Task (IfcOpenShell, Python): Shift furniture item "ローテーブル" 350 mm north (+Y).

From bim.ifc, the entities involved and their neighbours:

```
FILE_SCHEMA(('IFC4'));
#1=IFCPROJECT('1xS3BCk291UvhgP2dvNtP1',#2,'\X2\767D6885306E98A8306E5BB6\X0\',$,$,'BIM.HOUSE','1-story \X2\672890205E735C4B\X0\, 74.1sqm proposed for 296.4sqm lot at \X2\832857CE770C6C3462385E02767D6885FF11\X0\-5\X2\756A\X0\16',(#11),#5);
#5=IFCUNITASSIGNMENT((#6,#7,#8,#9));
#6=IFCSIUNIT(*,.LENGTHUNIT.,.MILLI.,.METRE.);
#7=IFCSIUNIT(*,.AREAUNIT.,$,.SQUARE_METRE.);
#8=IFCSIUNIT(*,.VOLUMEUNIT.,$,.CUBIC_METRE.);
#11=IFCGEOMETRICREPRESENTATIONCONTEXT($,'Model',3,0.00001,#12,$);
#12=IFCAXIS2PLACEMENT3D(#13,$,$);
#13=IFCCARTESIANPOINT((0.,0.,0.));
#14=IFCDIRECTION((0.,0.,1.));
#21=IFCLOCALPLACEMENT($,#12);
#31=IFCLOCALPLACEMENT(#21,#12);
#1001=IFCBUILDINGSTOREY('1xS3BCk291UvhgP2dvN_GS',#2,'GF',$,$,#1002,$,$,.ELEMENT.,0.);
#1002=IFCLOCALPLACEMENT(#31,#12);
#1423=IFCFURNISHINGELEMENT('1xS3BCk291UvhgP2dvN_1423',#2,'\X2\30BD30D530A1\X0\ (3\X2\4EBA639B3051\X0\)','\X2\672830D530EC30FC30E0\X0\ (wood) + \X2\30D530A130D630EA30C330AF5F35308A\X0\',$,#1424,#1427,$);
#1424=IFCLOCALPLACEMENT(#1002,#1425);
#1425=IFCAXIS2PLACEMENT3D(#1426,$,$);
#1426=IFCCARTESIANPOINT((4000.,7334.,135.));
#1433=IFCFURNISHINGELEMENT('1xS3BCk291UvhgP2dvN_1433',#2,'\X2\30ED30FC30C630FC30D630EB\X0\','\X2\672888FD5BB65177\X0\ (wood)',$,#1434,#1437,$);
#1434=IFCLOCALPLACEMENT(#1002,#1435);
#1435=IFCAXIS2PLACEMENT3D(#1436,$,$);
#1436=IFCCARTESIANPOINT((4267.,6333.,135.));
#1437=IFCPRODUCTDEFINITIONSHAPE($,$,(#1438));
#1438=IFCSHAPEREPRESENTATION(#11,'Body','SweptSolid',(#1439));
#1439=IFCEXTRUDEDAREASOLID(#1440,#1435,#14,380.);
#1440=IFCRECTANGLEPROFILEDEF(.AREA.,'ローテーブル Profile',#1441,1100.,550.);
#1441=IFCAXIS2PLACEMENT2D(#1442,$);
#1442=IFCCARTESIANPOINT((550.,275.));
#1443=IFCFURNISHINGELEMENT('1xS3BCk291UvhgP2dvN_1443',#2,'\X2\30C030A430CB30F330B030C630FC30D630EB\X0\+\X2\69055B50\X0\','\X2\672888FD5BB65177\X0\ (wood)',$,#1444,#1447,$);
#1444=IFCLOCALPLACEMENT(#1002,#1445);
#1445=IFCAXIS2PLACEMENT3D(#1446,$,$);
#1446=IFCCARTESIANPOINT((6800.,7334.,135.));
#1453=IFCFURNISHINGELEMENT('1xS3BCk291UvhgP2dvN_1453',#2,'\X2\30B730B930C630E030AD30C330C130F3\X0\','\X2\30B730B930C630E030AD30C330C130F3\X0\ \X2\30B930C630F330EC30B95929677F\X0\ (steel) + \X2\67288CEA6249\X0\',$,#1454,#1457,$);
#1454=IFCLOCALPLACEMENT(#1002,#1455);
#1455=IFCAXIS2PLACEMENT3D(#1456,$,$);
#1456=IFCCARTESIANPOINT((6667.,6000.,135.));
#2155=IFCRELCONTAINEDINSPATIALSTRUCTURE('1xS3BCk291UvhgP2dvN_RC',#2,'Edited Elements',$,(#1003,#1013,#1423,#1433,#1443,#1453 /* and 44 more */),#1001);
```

```python
import ifcopenshell
import ifcopenshell.api.geometry
import ifcopenshell.util.placement
import ifcopenshell.util.unit

model = ifcopenshell.open("bim.ifc")
unit_scale = ifcopenshell.util.unit.calculate_unit_scale(model)

item = model.by_guid("1xS3BCk291UvhgP2dvN_1433")
matrix = ifcopenshell.util.placement.get_local_placement(item.ObjectPlacement)
matrix[1, 3] += 0.35 / unit_scale
ifcopenshell.api.geometry.edit_object_placement(model, product=item, matrix=matrix, is_si=False)

print(ifcopenshell.util.placement.get_local_placement(item.ObjectPlacement).round(3) + 0.0)

model.write("bim_rev.ifc")
```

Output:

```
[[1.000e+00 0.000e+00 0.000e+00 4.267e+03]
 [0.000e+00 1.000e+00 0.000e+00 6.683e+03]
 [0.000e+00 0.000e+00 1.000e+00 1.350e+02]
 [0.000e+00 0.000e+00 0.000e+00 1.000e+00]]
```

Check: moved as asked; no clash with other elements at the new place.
